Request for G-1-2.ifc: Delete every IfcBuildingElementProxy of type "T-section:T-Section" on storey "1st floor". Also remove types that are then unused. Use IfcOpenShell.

First a look at what the model holds.

```python
import ifcopenshell
import ifcopenshell.util.element

model = ifcopenshell.open("G-1-2.ifc")
print(model.schema)
storey = next(s for s in model.by_type("IfcBuildingStorey") if s.Name == "1st floor")
proxies = [e for e in ifcopenshell.util.element.get_decomposition(storey) if e.is_a("IfcBuildingElementProxy")]
seen = {}
for e in proxies:
    element_type = ifcopenshell.util.element.get_type(e)
    name = element_type.Name if element_type not in (None, e) else None
    seen[name] = seen.get(name, 0) + 1
for name, count in sorted(seen.items(), key=str):
    print(count, "x", name)
```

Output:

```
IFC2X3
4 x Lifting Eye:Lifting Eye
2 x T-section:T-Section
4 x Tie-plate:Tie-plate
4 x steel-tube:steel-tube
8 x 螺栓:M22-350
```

```python
import ifcopenshell
import ifcopenshell.api.root
import ifcopenshell.util.element

model = ifcopenshell.open("G-1-2.ifc")

storey = next(s for s in model.by_type("IfcBuildingStorey") if s.Name == "1st floor")
proxies = [e for e in ifcopenshell.util.element.get_decomposition(storey) if e.is_a("IfcBuildingElementProxy")]
targets = [e for e in proxies if (t := ifcopenshell.util.element.get_type(e)) not in (None, e) and t.Name == "T-section:T-Section"]
types = {ifcopenshell.util.element.get_type(e) for e in targets} - {None, *targets}

for e in targets:
    ifcopenshell.api.root.remove_product(model, product=e)
print(len(targets), "removed")

unused = [t for t in types if not ifcopenshell.util.element.get_types(t)]
for t in unused:
    ifcopenshell.api.root.remove_product(model, product=t)
print(len(unused), "unused types removed")

model.write("G-1-2_updated.ifc")
```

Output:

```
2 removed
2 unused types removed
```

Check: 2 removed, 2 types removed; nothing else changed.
